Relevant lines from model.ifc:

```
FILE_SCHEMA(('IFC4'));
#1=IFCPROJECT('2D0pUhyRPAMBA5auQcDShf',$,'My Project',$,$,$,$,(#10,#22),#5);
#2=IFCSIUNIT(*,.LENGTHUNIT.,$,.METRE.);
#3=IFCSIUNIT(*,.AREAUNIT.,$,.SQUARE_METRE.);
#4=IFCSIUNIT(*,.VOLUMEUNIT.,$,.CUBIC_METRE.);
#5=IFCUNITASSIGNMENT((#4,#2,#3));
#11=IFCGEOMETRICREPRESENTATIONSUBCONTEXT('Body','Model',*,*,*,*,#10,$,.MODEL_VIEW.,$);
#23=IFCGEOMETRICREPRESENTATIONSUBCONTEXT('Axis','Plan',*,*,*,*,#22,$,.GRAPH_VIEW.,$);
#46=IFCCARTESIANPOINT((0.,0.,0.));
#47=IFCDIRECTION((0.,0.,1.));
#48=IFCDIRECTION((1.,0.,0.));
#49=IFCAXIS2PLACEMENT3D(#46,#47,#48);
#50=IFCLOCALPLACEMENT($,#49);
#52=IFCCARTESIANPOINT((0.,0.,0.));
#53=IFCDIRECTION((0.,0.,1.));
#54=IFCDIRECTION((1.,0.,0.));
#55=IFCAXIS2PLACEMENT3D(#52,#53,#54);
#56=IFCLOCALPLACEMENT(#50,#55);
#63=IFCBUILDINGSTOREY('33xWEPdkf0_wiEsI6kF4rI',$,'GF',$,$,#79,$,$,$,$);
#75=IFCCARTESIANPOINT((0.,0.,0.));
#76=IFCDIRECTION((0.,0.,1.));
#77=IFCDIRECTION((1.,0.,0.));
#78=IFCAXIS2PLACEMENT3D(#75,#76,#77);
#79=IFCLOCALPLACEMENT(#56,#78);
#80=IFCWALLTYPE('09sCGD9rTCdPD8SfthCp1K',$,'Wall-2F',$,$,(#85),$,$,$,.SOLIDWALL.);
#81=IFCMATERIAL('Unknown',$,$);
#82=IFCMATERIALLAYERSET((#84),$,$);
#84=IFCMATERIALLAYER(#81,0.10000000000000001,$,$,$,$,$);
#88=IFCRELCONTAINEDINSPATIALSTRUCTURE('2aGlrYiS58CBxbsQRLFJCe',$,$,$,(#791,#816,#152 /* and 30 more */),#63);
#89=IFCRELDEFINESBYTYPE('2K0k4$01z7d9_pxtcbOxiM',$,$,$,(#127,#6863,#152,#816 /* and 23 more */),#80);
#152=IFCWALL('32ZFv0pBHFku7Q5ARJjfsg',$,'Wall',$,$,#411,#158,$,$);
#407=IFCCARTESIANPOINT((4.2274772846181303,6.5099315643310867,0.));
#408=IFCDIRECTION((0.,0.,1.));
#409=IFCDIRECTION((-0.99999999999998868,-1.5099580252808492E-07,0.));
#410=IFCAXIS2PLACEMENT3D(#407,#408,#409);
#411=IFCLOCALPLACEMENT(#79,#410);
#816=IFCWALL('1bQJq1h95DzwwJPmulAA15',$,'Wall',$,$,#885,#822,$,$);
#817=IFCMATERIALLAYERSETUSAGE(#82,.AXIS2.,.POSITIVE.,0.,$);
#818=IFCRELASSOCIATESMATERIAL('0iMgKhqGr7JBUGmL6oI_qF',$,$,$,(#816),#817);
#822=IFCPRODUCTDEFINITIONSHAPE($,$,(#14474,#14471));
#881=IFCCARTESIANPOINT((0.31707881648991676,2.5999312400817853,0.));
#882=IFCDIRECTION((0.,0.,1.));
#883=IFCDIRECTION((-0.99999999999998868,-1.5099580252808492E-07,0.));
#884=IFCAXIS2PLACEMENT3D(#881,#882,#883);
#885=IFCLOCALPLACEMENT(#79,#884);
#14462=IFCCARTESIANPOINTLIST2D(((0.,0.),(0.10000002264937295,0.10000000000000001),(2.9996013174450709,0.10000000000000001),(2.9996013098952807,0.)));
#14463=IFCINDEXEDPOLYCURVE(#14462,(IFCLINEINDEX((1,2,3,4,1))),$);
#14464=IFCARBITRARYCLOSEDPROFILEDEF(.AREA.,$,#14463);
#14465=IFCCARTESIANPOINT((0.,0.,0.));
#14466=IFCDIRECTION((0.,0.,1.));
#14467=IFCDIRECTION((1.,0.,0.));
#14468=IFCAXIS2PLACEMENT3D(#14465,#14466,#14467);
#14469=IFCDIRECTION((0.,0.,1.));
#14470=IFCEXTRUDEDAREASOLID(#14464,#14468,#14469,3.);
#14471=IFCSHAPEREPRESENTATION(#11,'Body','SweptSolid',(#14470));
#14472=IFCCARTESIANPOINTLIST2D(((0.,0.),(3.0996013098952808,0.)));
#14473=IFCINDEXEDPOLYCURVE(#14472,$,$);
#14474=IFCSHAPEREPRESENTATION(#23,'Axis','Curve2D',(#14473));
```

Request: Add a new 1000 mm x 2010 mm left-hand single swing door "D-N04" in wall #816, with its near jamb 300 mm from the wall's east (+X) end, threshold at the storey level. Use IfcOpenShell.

```python
import numpy as np
import ifcopenshell
import ifcopenshell.api.feature
import ifcopenshell.api.geometry
import ifcopenshell.api.root
import ifcopenshell.api.spatial
import ifcopenshell.geom
import ifcopenshell.util.element
import ifcopenshell.util.placement
import ifcopenshell.util.representation
import ifcopenshell.util.shape
import ifcopenshell.util.unit

model = ifcopenshell.open("model.ifc")
unit_scale = ifcopenshell.util.unit.calculate_unit_scale(model)
settings = ifcopenshell.geom.settings()


def volume(element):
    """Net volume in cubic metres, openings subtracted."""
    shape = ifcopenshell.geom.create_shape(settings, element)
    return ifcopenshell.util.shape.get_volume(shape.geometry)


wall = model.by_guid("1bQJq1h95DzwwJPmulAA15")
storey = ifcopenshell.util.element.get_container(wall, ifc_class="IfcBuildingStorey")
context = ifcopenshell.util.representation.get_context(model, "Model", "Body", "MODEL_VIEW")
before = volume(wall)

width, height, from_end, sill = 1, 2.01, 0.3, 0.0  # metres

# The wall runs along its own X axis, and the end named is its -X end.
wall_shape = ifcopenshell.geom.create_shape(settings, wall)
x, y, z = ifcopenshell.util.shape.get_vertices(wall_shape.geometry).T
start = x.min() + from_end
face, thickness = float(y.min()), float(y.max() - y.min())
wall_matrix = ifcopenshell.util.placement.get_local_placement(wall.ObjectPlacement)
level = ifcopenshell.util.placement.get_local_placement(storey.ObjectPlacement)[2, 3]


def in_wall(x, y):
    """Placement at x, y metres in the wall's axes, at sill height."""
    matrix = wall_matrix.copy()
    matrix[:, 3] = wall_matrix @ np.array([x / unit_scale, y / unit_scale, 0.0, 1.0])
    matrix[2, 3] = level + sill / unit_scale
    return matrix


# Opening: a box that overshoots both wall faces by 50 mm.
opening = ifcopenshell.api.root.create_entity(model, ifc_class="IfcOpeningElement", predefined_type="OPENING")
box = ifcopenshell.api.geometry.add_wall_representation(
    model, context=context, length=width, height=height, thickness=thickness + 0.1
)
ifcopenshell.api.geometry.assign_representation(model, product=opening, representation=box)
ifcopenshell.api.geometry.edit_object_placement(model, product=opening, matrix=in_wall(start, face - 0.05), is_si=False)
ifcopenshell.api.feature.add_feature(model, feature=opening, element=wall)

door = ifcopenshell.api.root.create_entity(model, ifc_class="IfcDoor", name="D-N04", predefined_type="DOOR")
door.OverallWidth, door.OverallHeight = width / unit_scale, height / unit_scale
door.OperationType = "SINGLE_SWING_LEFT"
body = ifcopenshell.api.geometry.add_door_representation(
    model,
    context=context,
    overall_width=door.OverallWidth,
    overall_height=door.OverallHeight,
    operation_type="SINGLE_SWING_LEFT",
    lining_properties={"LiningDepth": thickness / unit_scale, "ThresholdDepth": thickness / unit_scale},
)
ifcopenshell.api.geometry.assign_representation(model, product=door, representation=body)
ifcopenshell.api.spatial.assign_container(model, products=[door], relating_structure=storey)
ifcopenshell.api.feature.add_filling(model, opening=opening, element=door)

# The lining spans the wall, so the door starts at the wall face.
ifcopenshell.api.geometry.edit_object_placement(model, product=door, matrix=in_wall(start, face), is_si=False)

after = volume(wall)

print(f"wall volume {before:.3f} -> {after:.3f} m3")

model.write("model-out.ifc")
```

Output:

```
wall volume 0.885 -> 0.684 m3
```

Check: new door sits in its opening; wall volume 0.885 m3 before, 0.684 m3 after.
